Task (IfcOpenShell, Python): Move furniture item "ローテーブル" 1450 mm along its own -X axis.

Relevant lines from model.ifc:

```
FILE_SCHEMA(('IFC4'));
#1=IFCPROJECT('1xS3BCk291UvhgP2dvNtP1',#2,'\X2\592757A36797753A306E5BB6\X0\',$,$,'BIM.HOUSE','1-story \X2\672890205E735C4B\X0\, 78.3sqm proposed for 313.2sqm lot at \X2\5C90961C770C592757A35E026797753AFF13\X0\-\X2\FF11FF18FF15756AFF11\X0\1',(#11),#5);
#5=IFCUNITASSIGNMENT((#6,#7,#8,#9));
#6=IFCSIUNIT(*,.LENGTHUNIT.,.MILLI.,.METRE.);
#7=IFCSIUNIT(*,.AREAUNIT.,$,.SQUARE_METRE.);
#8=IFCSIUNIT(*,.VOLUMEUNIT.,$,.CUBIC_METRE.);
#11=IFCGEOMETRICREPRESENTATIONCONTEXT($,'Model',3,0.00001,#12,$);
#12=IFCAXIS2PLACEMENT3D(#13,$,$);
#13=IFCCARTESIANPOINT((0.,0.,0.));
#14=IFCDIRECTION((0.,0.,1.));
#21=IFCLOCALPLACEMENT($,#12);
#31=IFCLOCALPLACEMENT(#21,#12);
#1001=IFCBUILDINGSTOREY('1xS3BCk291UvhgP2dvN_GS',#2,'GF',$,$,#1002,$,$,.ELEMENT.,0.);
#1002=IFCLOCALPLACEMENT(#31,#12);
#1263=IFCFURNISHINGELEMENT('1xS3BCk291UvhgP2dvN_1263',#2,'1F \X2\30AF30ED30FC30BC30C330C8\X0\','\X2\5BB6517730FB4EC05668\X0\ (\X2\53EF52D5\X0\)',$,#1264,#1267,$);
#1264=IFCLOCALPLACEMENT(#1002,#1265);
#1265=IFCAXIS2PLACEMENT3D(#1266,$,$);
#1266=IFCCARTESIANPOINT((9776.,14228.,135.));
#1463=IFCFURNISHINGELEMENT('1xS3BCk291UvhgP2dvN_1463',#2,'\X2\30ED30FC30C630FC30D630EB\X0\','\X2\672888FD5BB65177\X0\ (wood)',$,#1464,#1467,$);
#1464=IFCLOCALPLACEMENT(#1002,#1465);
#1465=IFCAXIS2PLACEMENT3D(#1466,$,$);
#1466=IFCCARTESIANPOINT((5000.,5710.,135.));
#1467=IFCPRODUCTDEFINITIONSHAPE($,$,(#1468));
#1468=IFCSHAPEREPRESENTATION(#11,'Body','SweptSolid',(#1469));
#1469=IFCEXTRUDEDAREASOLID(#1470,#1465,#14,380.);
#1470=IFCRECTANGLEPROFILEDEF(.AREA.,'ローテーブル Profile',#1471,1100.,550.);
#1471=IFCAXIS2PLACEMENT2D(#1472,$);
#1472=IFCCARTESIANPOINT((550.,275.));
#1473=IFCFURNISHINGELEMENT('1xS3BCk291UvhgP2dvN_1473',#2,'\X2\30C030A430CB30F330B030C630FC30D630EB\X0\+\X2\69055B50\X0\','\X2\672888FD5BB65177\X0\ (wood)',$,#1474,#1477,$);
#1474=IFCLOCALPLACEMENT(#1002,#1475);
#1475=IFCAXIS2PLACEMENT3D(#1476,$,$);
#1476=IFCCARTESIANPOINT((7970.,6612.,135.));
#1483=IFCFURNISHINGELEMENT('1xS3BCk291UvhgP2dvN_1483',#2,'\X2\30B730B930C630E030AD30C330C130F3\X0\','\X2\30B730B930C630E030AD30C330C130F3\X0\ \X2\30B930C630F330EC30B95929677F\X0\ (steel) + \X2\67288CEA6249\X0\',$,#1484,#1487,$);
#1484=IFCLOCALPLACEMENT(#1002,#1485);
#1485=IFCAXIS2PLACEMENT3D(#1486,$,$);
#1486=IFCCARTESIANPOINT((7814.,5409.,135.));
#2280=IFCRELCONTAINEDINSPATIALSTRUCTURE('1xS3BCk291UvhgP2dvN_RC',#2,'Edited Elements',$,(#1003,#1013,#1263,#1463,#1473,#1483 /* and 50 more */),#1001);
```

```python
import ifcopenshell
import ifcopenshell.api.geometry
import ifcopenshell.util.placement

model = ifcopenshell.open("model.ifc")

item = model.by_guid("1xS3BCk291UvhgP2dvN_1463")
matrix = ifcopenshell.util.placement.get_local_placement(item.ObjectPlacement)
matrix[:3, 3] -= matrix[:3, 0] * 1450.0
ifcopenshell.api.geometry.edit_object_placement(model, product=item, matrix=matrix, is_si=False)

print(ifcopenshell.util.placement.get_local_placement(item.ObjectPlacement).round(3) + 0.0)

model.write("model_updated.ifc")
```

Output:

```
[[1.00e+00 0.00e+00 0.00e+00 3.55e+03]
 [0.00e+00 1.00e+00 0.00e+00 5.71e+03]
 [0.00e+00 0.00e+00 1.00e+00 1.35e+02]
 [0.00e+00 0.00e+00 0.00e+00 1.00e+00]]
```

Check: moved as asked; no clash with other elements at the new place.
